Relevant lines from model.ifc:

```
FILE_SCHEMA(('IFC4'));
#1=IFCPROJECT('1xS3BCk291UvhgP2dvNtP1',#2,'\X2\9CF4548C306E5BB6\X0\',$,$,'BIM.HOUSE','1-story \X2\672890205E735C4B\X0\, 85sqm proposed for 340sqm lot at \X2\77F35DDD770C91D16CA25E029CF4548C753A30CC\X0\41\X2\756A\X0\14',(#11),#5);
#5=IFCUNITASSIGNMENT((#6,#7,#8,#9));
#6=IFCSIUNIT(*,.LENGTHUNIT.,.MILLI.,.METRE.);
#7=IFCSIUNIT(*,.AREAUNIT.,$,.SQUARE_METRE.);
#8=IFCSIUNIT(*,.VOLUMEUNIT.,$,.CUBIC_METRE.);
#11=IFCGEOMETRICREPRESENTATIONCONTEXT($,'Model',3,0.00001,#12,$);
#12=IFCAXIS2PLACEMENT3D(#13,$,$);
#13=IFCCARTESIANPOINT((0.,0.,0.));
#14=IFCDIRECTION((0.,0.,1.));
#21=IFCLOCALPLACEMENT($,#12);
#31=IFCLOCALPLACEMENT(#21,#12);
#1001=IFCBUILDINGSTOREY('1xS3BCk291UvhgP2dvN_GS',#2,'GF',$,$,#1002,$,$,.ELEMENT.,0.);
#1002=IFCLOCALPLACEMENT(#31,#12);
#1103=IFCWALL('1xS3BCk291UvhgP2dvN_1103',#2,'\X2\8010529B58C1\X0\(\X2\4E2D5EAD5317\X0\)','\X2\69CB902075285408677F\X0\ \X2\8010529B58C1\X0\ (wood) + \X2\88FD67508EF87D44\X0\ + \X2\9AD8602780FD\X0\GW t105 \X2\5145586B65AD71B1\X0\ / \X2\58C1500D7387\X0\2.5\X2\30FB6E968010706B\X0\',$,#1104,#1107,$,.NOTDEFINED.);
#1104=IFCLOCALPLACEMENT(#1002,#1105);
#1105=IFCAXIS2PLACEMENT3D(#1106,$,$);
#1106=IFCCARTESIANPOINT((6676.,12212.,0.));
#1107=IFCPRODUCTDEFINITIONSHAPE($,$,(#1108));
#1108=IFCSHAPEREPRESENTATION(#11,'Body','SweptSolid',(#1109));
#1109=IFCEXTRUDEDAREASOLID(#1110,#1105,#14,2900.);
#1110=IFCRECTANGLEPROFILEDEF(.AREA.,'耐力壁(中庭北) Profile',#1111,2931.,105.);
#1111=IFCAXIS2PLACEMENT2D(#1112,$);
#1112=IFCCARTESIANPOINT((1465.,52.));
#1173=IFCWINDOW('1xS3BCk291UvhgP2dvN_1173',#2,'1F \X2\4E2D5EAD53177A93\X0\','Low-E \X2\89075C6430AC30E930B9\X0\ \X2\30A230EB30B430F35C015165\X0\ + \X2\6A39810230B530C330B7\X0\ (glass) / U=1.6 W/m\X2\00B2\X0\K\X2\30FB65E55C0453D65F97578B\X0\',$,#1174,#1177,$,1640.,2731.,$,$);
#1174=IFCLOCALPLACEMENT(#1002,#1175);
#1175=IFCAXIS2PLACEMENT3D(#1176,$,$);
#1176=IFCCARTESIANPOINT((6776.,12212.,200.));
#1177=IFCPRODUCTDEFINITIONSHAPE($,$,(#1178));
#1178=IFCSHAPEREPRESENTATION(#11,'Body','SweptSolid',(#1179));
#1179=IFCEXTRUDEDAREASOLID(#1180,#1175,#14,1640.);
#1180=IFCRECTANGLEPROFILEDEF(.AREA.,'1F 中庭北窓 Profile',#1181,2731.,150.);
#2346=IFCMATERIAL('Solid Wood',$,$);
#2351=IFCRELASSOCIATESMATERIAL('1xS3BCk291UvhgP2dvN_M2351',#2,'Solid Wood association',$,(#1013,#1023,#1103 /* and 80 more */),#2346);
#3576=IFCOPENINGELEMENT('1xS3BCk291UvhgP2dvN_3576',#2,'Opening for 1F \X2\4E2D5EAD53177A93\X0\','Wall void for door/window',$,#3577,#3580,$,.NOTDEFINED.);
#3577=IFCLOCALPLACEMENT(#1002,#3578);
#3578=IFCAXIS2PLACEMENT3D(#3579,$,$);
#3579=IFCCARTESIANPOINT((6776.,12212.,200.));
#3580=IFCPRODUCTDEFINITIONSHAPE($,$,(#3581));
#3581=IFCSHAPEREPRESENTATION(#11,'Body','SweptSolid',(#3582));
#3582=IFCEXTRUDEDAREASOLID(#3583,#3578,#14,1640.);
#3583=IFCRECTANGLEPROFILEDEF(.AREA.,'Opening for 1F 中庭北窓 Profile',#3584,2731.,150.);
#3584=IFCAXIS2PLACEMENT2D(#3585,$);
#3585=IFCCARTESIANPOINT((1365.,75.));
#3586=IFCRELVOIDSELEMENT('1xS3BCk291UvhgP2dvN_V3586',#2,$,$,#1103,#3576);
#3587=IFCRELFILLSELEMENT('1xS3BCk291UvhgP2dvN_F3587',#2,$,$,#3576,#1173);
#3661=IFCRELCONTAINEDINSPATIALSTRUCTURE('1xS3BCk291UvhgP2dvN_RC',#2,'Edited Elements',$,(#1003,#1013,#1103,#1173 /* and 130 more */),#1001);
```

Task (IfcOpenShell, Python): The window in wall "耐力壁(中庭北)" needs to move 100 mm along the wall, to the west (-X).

```python
import ifcopenshell
import ifcopenshell.api.geometry
import ifcopenshell.util.placement
import ifcopenshell.util.unit

model = ifcopenshell.open("model.ifc")
unit_scale = ifcopenshell.util.unit.calculate_unit_scale(model)

window = model.by_id(1173)
opening = window.FillsVoids[0].RelatingOpeningElement
wall = opening.VoidsElements[0].RelatingBuildingElement

wall_matrix = ifcopenshell.util.placement.get_local_placement(wall.ObjectPlacement)
shift = wall_matrix[:3, 0] * -0.1 / unit_scale
before = ifcopenshell.util.placement.get_local_placement(window.ObjectPlacement)[:3, 3].copy()

# The window is not placed relative to its opening, so move both.
for product in (opening, window):
    matrix = ifcopenshell.util.placement.get_local_placement(product.ObjectPlacement)
    matrix[:3, 3] += shift
    ifcopenshell.api.geometry.edit_object_placement(model, product=product, matrix=matrix, is_si=False)

after = ifcopenshell.util.placement.get_local_placement(window.ObjectPlacement)[:3, 3]
print("window moved by", (after - before).round(3) + 0.0)

model.write("model_v2.ifc")
```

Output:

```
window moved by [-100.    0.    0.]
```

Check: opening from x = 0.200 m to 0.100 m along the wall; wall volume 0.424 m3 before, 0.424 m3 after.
